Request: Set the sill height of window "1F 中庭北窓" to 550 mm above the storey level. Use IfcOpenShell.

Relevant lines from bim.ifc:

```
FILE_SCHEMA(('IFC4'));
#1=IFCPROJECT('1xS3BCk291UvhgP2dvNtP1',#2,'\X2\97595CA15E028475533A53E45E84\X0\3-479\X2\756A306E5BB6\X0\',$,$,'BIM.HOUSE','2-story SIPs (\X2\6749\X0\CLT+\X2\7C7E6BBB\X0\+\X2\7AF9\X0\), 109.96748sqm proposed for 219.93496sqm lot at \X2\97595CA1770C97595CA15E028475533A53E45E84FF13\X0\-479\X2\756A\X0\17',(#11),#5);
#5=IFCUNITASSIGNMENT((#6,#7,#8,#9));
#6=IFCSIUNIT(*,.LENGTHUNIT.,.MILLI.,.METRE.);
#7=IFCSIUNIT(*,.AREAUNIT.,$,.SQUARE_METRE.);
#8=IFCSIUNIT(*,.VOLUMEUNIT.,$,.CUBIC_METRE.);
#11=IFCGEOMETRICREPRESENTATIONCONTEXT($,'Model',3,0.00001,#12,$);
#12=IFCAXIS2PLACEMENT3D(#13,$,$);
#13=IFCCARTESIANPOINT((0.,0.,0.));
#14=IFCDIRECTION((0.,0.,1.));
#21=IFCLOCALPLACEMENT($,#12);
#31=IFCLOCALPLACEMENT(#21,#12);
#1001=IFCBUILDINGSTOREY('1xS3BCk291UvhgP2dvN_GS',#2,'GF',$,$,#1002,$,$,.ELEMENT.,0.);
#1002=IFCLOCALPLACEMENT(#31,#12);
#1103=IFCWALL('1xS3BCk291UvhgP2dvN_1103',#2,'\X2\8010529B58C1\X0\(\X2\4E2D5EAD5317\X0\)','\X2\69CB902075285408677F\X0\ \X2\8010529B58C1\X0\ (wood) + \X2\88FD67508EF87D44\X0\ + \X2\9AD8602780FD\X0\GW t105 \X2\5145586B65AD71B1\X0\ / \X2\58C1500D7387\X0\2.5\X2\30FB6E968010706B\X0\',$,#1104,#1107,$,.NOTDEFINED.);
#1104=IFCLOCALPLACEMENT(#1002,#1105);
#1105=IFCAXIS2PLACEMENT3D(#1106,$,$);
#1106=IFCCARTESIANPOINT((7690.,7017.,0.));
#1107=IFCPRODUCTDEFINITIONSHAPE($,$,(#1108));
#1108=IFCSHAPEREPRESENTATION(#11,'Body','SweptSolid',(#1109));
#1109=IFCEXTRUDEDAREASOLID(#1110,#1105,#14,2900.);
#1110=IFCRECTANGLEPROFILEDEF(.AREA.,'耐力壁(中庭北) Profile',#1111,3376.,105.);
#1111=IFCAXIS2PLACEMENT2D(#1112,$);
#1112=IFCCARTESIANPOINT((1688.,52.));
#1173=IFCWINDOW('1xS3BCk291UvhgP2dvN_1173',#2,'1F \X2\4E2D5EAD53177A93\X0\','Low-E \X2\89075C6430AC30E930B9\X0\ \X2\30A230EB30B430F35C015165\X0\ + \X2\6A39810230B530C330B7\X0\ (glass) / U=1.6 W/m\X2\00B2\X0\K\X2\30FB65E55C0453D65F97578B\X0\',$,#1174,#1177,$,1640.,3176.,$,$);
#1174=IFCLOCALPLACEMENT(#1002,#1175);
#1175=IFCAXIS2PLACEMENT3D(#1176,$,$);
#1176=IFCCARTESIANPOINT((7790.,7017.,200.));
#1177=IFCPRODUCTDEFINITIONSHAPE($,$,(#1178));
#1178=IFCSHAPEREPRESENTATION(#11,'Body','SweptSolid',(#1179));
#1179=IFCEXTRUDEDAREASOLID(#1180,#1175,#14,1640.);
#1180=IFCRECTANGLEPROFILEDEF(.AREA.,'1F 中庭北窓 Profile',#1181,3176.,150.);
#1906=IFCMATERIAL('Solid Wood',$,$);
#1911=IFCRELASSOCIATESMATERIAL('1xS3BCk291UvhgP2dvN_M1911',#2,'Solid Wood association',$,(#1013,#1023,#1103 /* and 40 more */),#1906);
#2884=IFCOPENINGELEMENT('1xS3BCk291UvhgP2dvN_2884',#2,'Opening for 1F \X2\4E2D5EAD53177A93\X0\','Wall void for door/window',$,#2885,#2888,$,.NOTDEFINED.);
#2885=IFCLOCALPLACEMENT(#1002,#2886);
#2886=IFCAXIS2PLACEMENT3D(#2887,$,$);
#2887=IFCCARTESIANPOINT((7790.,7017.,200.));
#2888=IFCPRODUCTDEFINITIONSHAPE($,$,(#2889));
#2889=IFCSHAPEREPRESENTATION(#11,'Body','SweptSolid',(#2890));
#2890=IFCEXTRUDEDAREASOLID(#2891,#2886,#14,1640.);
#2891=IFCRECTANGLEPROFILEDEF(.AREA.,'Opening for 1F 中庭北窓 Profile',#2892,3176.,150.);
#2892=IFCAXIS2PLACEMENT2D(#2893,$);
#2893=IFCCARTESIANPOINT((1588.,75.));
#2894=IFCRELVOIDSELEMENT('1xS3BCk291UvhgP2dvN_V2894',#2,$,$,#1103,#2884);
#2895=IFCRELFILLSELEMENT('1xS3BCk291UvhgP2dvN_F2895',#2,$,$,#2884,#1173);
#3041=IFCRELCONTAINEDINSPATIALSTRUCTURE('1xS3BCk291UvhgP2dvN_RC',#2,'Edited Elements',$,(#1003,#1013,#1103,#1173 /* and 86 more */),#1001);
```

```python
import numpy as np
import ifcopenshell
import ifcopenshell.api.geometry
import ifcopenshell.geom
import ifcopenshell.util.element
import ifcopenshell.util.placement
import ifcopenshell.util.shape
import ifcopenshell.util.unit

model = ifcopenshell.open("bim.ifc")
unit_scale = ifcopenshell.util.unit.calculate_unit_scale(model)

window = model.by_guid("1xS3BCk291UvhgP2dvN_1173")
opening = window.FillsVoids[0].RelatingOpeningElement
storey = ifcopenshell.util.element.get_container(window, ifc_class="IfcBuildingStorey")
level = ifcopenshell.util.placement.get_local_placement(storey.ObjectPlacement)[2, 3]

# The opening's origin need not be at the sill, so measure its lowest point.
shape = ifcopenshell.geom.create_shape(ifcopenshell.geom.settings(), opening)
bottom = ifcopenshell.util.shape.get_shape_bottom_elevation(shape, shape.geometry) / unit_scale
dz = level + 550.0 - bottom

shift = np.array([0.0, 0.0, dz])
# The window is not placed relative to its opening, so move both.
for product in (opening, window):
    matrix = ifcopenshell.util.placement.get_local_placement(product.ObjectPlacement)
    matrix[:3, 3] += shift
    ifcopenshell.api.geometry.edit_object_placement(model, product=product, matrix=matrix, is_si=False)

print(f"moved by {dz * unit_scale:+.3f} m")

model.write("bim-out.ifc")
```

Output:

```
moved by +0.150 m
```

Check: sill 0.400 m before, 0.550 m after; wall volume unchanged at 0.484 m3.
